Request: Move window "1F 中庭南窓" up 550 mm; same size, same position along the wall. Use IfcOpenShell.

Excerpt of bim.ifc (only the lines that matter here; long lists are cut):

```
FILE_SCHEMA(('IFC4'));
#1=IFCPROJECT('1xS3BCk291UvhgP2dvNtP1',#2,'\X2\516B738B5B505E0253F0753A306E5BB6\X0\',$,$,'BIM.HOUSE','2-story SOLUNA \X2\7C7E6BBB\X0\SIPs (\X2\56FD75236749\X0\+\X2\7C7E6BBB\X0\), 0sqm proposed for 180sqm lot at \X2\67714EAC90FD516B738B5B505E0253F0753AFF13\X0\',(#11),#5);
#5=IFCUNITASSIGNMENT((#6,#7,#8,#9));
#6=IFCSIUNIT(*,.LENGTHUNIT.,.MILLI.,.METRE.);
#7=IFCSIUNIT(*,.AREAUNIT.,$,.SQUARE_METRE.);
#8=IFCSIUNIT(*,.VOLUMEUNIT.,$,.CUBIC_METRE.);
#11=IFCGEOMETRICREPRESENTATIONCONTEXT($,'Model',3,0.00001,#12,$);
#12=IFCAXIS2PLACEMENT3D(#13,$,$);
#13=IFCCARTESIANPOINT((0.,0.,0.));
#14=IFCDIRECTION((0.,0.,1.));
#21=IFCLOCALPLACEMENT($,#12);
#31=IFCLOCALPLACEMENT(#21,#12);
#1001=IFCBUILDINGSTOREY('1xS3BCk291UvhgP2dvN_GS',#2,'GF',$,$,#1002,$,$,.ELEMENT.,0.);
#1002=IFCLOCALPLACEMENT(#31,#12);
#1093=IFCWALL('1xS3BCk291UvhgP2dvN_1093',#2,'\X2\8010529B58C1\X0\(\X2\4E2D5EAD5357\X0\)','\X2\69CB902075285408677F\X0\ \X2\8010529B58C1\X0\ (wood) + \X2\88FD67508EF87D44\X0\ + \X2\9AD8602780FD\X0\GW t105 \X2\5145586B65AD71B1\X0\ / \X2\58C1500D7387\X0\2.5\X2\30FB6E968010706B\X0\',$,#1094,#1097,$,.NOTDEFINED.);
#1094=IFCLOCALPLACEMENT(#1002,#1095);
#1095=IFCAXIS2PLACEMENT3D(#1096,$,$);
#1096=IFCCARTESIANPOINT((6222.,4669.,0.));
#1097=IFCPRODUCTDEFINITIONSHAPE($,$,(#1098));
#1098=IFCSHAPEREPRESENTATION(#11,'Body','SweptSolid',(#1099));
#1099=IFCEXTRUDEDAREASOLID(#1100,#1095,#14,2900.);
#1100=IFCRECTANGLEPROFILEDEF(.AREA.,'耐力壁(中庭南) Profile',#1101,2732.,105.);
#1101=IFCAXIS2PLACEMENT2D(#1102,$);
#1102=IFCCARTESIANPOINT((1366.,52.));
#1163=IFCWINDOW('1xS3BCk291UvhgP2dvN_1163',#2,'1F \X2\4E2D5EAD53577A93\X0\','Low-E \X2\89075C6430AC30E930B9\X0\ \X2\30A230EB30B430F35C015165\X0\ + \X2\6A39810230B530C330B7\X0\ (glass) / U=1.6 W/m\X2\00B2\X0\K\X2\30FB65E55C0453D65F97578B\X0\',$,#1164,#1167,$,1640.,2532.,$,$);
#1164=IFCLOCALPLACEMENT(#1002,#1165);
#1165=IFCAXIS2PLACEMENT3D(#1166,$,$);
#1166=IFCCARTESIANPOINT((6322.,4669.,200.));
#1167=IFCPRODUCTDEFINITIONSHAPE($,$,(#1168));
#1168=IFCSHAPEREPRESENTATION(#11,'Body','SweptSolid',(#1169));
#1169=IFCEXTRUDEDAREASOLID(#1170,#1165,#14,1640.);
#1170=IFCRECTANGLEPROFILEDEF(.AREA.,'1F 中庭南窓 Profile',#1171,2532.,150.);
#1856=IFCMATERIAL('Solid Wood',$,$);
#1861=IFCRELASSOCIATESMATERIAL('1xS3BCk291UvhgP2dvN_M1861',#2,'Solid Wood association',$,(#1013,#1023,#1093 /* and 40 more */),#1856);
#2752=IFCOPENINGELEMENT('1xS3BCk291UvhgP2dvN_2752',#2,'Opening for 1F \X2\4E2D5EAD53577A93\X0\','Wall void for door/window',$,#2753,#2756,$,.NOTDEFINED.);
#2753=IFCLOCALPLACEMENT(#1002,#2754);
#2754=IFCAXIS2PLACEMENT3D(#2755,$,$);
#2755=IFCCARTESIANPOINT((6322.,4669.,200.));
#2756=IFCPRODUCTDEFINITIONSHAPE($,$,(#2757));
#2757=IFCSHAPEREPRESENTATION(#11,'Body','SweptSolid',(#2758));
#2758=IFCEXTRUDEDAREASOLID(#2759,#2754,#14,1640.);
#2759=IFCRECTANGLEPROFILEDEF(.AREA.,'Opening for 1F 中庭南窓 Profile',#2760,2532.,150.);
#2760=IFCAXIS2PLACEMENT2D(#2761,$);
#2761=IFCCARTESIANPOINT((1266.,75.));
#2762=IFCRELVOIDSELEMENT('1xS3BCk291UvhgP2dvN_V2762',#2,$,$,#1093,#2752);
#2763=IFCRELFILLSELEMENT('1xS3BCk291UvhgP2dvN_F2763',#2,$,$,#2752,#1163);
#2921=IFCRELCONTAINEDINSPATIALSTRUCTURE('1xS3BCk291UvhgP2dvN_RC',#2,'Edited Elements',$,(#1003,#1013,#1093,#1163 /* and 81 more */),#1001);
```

```python
import numpy as np
import ifcopenshell
import ifcopenshell.api.geometry
import ifcopenshell.util.placement
import ifcopenshell.util.unit

model = ifcopenshell.open("bim.ifc")
unit_scale = ifcopenshell.util.unit.calculate_unit_scale(model)

window = model.by_id(1163)
opening = window.FillsVoids[0].RelatingOpeningElement
dz = 550.0

shift = np.array([0.0, 0.0, dz])
# The window is not placed relative to its opening, so move both.
for product in (opening, window):
    matrix = ifcopenshell.util.placement.get_local_placement(product.ObjectPlacement)
    matrix[:3, 3] += shift
    ifcopenshell.api.geometry.edit_object_placement(model, product=product, matrix=matrix, is_si=False)

print(f"moved by {dz * unit_scale:+.3f} m")

model.write("bim-out.ifc")
```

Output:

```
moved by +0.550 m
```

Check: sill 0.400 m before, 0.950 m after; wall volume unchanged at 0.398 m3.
